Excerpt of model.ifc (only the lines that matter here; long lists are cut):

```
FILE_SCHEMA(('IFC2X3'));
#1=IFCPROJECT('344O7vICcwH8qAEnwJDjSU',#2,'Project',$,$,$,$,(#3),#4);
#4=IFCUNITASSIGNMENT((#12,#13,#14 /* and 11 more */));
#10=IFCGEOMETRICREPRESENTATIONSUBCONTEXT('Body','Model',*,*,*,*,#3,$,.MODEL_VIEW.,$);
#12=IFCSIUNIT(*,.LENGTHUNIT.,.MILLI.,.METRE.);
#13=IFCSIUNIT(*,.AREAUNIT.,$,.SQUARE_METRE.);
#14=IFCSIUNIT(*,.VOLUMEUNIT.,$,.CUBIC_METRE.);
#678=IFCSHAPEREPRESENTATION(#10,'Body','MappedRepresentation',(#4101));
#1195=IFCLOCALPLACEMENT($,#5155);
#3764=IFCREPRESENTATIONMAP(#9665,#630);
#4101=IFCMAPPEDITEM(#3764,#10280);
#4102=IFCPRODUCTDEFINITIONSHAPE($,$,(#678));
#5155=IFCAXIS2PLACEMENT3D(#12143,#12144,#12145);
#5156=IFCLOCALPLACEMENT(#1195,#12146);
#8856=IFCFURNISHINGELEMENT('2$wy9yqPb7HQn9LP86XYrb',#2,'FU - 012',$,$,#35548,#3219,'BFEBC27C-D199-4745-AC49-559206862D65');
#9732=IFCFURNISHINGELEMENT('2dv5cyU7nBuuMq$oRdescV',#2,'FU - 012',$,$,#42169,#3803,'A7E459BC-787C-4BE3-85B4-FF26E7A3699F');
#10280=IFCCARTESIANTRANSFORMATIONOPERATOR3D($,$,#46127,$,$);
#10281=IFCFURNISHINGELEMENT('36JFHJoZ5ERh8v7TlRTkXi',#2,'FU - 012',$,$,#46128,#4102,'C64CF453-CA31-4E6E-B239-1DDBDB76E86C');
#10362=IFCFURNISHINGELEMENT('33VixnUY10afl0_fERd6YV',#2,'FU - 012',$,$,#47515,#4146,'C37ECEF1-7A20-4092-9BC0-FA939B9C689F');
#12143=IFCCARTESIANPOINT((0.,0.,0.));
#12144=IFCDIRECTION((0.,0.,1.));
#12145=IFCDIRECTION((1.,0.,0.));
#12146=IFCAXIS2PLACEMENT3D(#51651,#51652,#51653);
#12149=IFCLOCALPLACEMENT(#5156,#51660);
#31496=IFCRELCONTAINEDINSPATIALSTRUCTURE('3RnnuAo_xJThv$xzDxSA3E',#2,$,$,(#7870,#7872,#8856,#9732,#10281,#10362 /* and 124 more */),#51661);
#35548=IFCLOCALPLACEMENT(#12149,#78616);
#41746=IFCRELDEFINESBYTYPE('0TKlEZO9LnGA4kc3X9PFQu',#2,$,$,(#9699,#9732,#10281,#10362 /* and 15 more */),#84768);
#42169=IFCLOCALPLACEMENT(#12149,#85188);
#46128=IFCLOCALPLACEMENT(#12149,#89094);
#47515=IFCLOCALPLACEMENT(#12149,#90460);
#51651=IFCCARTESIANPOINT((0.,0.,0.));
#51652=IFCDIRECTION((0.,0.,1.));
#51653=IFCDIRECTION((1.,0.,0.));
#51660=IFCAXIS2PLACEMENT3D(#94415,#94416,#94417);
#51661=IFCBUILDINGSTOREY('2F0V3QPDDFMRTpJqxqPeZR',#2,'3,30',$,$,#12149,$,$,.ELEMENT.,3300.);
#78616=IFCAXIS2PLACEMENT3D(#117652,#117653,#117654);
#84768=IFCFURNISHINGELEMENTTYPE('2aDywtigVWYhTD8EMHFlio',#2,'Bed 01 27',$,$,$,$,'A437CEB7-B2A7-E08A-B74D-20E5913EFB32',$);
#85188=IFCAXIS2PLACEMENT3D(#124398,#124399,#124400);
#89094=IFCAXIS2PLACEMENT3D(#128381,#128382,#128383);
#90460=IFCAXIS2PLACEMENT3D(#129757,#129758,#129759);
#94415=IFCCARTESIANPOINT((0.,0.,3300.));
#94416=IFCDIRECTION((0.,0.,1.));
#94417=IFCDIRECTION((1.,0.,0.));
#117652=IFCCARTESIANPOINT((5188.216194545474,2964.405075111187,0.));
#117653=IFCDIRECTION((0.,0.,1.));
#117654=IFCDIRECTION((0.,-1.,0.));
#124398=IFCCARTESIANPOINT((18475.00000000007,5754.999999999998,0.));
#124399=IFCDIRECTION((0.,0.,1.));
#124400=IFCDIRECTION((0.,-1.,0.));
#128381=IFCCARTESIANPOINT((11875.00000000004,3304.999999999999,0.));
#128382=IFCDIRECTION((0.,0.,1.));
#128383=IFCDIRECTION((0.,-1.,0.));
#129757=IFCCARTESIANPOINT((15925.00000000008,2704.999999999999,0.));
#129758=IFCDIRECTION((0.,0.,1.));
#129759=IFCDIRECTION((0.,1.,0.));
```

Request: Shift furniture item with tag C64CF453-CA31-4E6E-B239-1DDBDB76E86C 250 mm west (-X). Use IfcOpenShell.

```python
import ifcopenshell
import ifcopenshell.api.geometry
import ifcopenshell.util.placement
import ifcopenshell.util.unit

model = ifcopenshell.open("model.ifc")
unit_scale = ifcopenshell.util.unit.calculate_unit_scale(model)

item = model.by_guid("36JFHJoZ5ERh8v7TlRTkXi")
matrix = ifcopenshell.util.placement.get_local_placement(item.ObjectPlacement)
matrix[0, 3] -= 0.25 / unit_scale
ifcopenshell.api.geometry.edit_object_placement(model, product=item, matrix=matrix, is_si=False)

print(ifcopenshell.util.placement.get_local_placement(item.ObjectPlacement).round(3) + 0.0)

model.write("model-out.ifc")
```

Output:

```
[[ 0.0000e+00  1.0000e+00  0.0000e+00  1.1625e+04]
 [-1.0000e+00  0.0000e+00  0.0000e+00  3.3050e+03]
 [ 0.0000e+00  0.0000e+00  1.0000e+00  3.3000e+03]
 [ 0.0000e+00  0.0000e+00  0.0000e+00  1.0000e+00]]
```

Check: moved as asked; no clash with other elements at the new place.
